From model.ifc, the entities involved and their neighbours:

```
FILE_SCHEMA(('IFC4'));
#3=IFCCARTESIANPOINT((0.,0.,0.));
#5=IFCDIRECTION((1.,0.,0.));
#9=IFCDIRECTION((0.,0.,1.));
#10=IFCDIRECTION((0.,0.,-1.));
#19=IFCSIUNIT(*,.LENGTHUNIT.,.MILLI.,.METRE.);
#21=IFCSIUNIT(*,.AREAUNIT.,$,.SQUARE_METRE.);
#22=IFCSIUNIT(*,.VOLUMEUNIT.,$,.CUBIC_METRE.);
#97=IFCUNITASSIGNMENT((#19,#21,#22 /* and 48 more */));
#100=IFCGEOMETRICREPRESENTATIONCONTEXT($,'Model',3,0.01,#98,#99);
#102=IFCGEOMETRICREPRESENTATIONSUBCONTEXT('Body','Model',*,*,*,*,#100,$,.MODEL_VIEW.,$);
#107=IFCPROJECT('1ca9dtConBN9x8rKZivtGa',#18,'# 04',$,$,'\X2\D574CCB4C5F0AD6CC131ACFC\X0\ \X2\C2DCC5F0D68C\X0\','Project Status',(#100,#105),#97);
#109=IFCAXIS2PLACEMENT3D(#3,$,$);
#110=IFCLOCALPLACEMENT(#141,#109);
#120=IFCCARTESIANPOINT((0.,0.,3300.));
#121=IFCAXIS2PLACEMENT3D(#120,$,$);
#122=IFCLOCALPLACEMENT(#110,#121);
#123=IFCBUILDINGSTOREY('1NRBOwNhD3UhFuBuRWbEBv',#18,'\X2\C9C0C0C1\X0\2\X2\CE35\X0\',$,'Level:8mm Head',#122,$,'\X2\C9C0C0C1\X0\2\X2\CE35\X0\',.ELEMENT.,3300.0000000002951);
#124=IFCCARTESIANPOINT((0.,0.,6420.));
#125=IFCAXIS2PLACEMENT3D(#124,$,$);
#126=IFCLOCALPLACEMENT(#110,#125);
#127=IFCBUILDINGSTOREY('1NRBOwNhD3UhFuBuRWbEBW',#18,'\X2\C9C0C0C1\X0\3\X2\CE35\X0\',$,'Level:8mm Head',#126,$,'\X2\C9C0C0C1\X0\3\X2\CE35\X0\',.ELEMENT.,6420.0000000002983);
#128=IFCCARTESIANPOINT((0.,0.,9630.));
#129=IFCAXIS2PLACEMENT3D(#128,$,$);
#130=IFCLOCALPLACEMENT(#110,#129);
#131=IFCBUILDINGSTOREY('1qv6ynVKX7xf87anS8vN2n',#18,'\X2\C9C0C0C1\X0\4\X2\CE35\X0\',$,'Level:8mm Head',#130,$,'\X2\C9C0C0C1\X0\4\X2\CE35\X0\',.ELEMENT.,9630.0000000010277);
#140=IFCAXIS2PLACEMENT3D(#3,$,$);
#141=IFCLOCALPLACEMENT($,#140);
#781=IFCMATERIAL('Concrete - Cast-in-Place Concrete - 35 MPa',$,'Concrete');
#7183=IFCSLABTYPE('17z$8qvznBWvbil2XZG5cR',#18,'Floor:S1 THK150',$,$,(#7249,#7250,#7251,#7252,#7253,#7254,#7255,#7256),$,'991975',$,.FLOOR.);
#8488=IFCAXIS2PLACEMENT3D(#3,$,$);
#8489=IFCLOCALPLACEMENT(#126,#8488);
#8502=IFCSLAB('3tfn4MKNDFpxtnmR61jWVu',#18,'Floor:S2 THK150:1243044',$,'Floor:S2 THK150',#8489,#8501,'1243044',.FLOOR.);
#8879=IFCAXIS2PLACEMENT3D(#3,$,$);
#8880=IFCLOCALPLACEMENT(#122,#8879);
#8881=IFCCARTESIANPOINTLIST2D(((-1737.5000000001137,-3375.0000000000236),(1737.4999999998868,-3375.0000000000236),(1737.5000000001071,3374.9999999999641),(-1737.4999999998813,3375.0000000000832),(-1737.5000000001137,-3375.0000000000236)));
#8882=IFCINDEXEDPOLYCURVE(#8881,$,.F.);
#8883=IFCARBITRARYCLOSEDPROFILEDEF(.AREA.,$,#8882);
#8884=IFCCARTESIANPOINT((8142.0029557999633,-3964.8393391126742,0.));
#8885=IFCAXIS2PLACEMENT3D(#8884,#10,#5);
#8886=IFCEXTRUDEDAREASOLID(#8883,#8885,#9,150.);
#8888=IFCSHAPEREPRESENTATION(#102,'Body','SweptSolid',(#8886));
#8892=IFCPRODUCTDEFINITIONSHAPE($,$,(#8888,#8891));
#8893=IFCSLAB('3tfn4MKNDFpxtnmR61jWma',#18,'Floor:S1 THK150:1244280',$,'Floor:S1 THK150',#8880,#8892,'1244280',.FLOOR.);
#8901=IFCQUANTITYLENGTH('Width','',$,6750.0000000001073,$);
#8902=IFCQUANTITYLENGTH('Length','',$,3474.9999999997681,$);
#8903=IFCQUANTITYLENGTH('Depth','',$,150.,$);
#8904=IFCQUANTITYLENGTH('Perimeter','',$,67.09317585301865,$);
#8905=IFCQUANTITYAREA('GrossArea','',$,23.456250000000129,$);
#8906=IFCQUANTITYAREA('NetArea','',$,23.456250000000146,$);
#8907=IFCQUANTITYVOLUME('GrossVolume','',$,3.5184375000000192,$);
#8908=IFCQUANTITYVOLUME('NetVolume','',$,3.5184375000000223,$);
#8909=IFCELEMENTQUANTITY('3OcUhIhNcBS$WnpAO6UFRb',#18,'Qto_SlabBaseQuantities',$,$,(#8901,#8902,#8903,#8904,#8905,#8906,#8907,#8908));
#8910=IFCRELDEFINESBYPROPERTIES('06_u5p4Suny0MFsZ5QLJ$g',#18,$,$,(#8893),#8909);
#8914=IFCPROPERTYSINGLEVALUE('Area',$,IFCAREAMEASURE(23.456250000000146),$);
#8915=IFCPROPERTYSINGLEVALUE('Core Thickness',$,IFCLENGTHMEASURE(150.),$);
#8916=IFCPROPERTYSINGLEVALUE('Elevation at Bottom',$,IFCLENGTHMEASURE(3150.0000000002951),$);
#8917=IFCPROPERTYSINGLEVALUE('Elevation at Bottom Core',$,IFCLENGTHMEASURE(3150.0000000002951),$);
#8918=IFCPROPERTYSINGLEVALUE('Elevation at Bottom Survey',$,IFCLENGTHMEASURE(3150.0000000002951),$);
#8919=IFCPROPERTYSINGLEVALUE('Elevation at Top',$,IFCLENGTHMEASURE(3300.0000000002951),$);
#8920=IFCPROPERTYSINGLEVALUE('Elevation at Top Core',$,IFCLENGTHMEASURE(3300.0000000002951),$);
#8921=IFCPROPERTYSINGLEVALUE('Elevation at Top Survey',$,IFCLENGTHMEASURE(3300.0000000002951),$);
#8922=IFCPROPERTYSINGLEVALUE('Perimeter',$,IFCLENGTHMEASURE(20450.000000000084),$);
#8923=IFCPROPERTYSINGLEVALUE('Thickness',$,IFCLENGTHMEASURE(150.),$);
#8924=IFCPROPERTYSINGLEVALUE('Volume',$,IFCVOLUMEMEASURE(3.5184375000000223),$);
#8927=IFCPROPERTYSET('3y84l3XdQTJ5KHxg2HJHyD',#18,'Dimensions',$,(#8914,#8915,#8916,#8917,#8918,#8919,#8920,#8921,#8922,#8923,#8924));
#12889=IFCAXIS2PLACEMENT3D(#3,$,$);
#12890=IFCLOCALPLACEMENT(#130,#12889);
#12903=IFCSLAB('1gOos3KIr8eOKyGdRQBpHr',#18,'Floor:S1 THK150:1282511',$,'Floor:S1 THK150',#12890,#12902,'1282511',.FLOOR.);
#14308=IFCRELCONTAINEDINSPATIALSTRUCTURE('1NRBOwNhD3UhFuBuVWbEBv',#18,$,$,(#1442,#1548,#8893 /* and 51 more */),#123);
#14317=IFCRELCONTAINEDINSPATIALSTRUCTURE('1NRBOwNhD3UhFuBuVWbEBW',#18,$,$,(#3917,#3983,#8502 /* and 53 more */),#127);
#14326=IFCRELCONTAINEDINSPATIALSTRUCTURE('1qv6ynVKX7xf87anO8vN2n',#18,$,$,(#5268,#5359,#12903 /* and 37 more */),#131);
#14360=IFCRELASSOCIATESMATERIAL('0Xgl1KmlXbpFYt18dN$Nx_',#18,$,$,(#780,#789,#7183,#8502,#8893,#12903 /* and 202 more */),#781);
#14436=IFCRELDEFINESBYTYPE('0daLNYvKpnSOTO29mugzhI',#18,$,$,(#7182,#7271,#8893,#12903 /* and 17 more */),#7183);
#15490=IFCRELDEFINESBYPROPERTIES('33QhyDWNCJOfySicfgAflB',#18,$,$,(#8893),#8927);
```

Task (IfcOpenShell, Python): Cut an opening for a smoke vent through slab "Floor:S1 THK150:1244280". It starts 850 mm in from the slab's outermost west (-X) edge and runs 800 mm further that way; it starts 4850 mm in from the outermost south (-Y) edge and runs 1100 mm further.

```python
import numpy as np
import ifcopenshell
import ifcopenshell.api.feature
import ifcopenshell.api.geometry
import ifcopenshell.api.pset
import ifcopenshell.api.root
import ifcopenshell.geom
import ifcopenshell.util.element
import ifcopenshell.util.placement
import ifcopenshell.util.representation
import ifcopenshell.util.shape
import ifcopenshell.util.unit

model = ifcopenshell.open("model.ifc")
unit_scale = ifcopenshell.util.unit.calculate_unit_scale(model)
area_scale = ifcopenshell.util.unit.calculate_unit_scale(model, "AREAUNIT")
volume_scale = ifcopenshell.util.unit.calculate_unit_scale(model, "VOLUMEUNIT")
settings = ifcopenshell.geom.settings()


def volume(element):
    """Net volume in cubic metres, openings subtracted."""
    shape = ifcopenshell.geom.create_shape(settings, element)
    return ifcopenshell.util.shape.get_volume(shape.geometry)


slab = model.by_guid("3tfn4MKNDFpxtnmR61jWma")
before = volume(slab)

# Extent in the slab's own axes, in metres. The edges named are its -X and -Y sides.
slab_shape = ifcopenshell.geom.create_shape(settings, slab)
vertices = ifcopenshell.util.shape.get_vertices(slab_shape.geometry)
x_min, y_min, bottom = vertices.min(axis=0)
top = vertices[:, 2].max()

opening = ifcopenshell.api.root.create_entity(model, ifc_class="IfcOpeningElement", name="Smoke vent opening", predefined_type="OPENING")
context = ifcopenshell.util.representation.get_context(model, "Model", "Body", "MODEL_VIEW")
width, depth = 0.8, 1.1
outline = [(0.0, 0.0), (width, 0.0), (width, depth), (0.0, depth), (0.0, 0.0)]
# Overshoot both faces by 50 mm so the cut is clean.
shape = ifcopenshell.api.geometry.add_slab_representation(
    model, context=context, depth=top - bottom + 0.1, polyline=outline
)
ifcopenshell.api.geometry.assign_representation(model, product=opening, representation=shape)

matrix = ifcopenshell.util.placement.get_local_placement(slab.ObjectPlacement)
matrix[:, 3] = matrix @ np.append(np.array([x_min + 0.85, y_min + 4.85, bottom - 0.05]) / unit_scale, 1.0)
ifcopenshell.api.geometry.edit_object_placement(model, product=opening, matrix=matrix, is_si=False)
ifcopenshell.api.feature.add_feature(model, feature=opening, element=slab)

after = volume(slab)

# Update the slab's stored quantities.
qto = model.by_id(ifcopenshell.util.element.get_pset(slab, "Qto_SlabBaseQuantities", should_inherit=False)["id"])
ifcopenshell.api.pset.edit_qto(model, qto=qto, properties={
    "NetArea": after / (top - bottom) / area_scale,
    "NetVolume": after / volume_scale,
})
pset = model.by_id(ifcopenshell.util.element.get_pset(slab, "Dimensions", should_inherit=False)["id"])
ifcopenshell.api.pset.edit_pset(model, pset=pset, properties={
    "Area": model.create_entity("IfcAreaMeasure", after / (top - bottom) / area_scale),
    "Volume": model.create_entity("IfcVolumeMeasure", after / volume_scale),
})

print(f"slab volume {before:.3f} -> {after:.3f} m3")

model.write("model_v2.ifc")
```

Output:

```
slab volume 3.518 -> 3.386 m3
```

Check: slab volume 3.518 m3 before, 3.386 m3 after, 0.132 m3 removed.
